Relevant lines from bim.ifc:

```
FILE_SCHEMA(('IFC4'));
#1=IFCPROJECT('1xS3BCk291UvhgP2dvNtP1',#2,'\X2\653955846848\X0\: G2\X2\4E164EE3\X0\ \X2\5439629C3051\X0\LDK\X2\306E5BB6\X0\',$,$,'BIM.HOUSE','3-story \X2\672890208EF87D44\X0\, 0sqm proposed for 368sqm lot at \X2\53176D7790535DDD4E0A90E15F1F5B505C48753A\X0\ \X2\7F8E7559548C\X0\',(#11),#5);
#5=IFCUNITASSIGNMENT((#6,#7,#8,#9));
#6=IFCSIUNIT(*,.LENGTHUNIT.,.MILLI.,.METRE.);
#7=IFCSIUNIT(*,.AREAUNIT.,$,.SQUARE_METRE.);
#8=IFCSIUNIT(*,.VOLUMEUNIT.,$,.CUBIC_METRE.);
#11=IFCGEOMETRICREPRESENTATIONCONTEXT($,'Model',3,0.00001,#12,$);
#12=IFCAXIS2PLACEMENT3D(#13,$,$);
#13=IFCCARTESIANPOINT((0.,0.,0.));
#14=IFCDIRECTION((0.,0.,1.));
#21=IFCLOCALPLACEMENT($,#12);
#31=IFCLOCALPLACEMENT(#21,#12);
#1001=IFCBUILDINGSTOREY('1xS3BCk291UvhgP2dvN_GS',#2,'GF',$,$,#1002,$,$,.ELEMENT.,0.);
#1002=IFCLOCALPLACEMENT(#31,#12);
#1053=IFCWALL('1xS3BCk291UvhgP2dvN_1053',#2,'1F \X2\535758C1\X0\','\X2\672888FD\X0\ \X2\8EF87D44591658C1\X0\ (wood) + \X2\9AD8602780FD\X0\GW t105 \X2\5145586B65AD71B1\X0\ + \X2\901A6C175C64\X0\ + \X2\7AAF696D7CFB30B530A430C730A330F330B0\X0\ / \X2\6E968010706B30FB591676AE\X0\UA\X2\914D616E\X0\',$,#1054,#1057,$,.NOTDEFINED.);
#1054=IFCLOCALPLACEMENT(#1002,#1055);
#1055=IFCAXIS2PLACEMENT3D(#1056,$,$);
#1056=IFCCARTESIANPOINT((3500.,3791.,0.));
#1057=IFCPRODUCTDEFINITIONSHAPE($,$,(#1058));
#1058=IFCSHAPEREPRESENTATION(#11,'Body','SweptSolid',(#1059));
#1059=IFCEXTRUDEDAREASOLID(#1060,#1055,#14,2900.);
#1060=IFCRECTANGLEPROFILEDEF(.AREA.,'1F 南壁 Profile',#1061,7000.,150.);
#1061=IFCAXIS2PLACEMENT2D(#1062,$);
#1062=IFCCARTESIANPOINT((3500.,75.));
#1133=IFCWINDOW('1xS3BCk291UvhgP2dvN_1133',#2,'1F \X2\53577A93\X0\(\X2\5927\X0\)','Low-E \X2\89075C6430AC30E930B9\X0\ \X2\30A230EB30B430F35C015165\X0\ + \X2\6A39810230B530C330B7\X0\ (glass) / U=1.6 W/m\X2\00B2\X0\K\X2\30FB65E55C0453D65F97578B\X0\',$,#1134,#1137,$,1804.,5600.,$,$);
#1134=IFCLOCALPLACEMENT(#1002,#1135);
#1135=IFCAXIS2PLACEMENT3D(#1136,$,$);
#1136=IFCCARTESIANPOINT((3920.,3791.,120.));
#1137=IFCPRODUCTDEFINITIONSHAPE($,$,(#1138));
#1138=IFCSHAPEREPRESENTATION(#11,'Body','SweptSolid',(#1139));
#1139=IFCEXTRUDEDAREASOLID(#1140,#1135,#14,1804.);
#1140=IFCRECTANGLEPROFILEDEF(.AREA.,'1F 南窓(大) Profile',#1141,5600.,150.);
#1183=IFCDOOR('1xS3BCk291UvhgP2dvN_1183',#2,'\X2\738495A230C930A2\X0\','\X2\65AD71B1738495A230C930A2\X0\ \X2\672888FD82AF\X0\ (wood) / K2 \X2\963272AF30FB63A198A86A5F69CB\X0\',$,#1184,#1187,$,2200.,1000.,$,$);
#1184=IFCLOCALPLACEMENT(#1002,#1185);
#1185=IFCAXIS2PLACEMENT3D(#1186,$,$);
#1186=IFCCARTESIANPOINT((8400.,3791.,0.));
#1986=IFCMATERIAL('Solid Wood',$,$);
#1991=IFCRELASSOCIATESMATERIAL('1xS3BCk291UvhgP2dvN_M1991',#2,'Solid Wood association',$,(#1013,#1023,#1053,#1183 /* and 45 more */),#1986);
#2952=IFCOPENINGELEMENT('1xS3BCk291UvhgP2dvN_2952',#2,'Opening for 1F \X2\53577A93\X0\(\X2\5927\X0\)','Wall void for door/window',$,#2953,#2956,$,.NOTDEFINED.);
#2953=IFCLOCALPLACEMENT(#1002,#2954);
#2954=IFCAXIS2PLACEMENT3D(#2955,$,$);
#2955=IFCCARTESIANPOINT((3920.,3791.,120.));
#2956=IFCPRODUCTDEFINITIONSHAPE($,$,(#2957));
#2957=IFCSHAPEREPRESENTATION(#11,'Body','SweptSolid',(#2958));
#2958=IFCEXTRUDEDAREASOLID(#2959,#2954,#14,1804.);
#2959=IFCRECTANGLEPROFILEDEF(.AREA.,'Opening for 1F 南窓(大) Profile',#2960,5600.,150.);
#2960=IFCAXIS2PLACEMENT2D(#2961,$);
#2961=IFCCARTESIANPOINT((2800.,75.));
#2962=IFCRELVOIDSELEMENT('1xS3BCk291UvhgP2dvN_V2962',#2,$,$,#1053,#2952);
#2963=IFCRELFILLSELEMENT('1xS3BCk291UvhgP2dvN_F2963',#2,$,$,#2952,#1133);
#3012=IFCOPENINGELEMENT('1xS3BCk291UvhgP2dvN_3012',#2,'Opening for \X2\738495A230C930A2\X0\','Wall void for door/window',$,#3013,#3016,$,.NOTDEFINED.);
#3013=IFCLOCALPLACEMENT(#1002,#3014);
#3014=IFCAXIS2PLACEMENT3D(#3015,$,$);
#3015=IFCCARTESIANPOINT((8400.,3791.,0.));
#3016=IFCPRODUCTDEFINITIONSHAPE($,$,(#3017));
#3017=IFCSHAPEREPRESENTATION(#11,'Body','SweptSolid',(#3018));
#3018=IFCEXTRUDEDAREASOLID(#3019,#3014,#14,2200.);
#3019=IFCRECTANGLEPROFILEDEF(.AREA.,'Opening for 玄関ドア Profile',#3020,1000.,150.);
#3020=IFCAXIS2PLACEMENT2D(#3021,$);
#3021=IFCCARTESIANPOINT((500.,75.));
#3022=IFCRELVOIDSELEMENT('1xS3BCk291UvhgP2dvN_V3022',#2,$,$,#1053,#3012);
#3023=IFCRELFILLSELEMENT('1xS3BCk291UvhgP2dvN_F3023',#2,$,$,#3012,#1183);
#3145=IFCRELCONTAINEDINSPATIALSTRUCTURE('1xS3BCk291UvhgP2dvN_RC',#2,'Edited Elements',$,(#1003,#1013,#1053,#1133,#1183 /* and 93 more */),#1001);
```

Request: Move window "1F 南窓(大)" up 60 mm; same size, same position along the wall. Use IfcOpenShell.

```python
import numpy as np
import ifcopenshell
import ifcopenshell.api.geometry
import ifcopenshell.util.placement
import ifcopenshell.util.unit

model = ifcopenshell.open("bim.ifc")
unit_scale = ifcopenshell.util.unit.calculate_unit_scale(model)

window = model.by_guid("1xS3BCk291UvhgP2dvN_1133")
opening = window.FillsVoids[0].RelatingOpeningElement
dz = 0.06 / unit_scale

shift = np.array([0.0, 0.0, dz])
# The window is not placed relative to its opening, so move both.
for product in (opening, window):
    matrix = ifcopenshell.util.placement.get_local_placement(product.ObjectPlacement)
    matrix[:3, 3] += shift
    ifcopenshell.api.geometry.edit_object_placement(model, product=product, matrix=matrix, is_si=False)

print(f"moved by {dz * unit_scale:+.3f} m")

model.write("bim_rev.ifc")
```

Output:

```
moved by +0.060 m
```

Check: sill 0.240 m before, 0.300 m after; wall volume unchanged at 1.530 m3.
